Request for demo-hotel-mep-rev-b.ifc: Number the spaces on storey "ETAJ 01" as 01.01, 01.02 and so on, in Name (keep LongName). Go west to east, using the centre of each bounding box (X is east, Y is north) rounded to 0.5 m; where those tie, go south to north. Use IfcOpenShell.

First a look at what the model holds.

```python
import ifcopenshell
import ifcopenshell.util.element
import ifcopenshell.util.placement

model = ifcopenshell.open("demo-hotel-mep-rev-b.ifc")
print(model.schema)
storey = next(s for s in model.by_type("IfcBuildingStorey") if s.Name == "ETAJ 01")
spaces = [e for e in ifcopenshell.util.element.get_decomposition(storey) if e.is_a("IfcSpace")]
for e in sorted(spaces, key=lambda e: e.id()):
    origin = ifcopenshell.util.placement.get_local_placement(e.ObjectPlacement)[:3, 3]
    print(e.id(), e.Name, e.LongName, origin.round(2) + 0.0, sep=" | ")
```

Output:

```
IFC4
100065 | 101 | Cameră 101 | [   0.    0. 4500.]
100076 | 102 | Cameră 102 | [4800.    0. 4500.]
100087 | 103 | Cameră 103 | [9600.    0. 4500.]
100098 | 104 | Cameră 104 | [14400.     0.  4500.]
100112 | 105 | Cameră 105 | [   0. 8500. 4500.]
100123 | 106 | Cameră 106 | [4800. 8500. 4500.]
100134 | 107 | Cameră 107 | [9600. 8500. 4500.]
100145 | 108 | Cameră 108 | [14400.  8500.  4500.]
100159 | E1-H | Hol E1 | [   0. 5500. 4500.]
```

```python
import ifcopenshell
import ifcopenshell.geom
import ifcopenshell.util.element
import ifcopenshell.util.shape

model = ifcopenshell.open("demo-hotel-mep-rev-b.ifc")
settings = ifcopenshell.geom.settings()
settings.set("use-world-coords", True)


def centre(element):
    shape = ifcopenshell.geom.create_shape(settings, element)
    return ifcopenshell.util.shape.get_bbox_centroid(shape.geometry)


storey = next(s for s in model.by_type("IfcBuildingStorey") if s.Name == "ETAJ 01")
spaces = [e for e in ifcopenshell.util.element.get_decomposition(storey) if e.is_a("IfcSpace")]

# Insertion points can sit at a corner or the storey origin, so sort by the geometry (in metres).
centres = {e: centre(e) for e in spaces}
spaces.sort(key=lambda e: (round(centres[e][0] / 0.5), centres[e][1]))

for i, e in enumerate(spaces, start=1):
    number = f"01.{i:02d}"
    e.Name = number
    print(e.id(), number)

model.write("demo-hotel-mep-rev-b-out.ifc")
```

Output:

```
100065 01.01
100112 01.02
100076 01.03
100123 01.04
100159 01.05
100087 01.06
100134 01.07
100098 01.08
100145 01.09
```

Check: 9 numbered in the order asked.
